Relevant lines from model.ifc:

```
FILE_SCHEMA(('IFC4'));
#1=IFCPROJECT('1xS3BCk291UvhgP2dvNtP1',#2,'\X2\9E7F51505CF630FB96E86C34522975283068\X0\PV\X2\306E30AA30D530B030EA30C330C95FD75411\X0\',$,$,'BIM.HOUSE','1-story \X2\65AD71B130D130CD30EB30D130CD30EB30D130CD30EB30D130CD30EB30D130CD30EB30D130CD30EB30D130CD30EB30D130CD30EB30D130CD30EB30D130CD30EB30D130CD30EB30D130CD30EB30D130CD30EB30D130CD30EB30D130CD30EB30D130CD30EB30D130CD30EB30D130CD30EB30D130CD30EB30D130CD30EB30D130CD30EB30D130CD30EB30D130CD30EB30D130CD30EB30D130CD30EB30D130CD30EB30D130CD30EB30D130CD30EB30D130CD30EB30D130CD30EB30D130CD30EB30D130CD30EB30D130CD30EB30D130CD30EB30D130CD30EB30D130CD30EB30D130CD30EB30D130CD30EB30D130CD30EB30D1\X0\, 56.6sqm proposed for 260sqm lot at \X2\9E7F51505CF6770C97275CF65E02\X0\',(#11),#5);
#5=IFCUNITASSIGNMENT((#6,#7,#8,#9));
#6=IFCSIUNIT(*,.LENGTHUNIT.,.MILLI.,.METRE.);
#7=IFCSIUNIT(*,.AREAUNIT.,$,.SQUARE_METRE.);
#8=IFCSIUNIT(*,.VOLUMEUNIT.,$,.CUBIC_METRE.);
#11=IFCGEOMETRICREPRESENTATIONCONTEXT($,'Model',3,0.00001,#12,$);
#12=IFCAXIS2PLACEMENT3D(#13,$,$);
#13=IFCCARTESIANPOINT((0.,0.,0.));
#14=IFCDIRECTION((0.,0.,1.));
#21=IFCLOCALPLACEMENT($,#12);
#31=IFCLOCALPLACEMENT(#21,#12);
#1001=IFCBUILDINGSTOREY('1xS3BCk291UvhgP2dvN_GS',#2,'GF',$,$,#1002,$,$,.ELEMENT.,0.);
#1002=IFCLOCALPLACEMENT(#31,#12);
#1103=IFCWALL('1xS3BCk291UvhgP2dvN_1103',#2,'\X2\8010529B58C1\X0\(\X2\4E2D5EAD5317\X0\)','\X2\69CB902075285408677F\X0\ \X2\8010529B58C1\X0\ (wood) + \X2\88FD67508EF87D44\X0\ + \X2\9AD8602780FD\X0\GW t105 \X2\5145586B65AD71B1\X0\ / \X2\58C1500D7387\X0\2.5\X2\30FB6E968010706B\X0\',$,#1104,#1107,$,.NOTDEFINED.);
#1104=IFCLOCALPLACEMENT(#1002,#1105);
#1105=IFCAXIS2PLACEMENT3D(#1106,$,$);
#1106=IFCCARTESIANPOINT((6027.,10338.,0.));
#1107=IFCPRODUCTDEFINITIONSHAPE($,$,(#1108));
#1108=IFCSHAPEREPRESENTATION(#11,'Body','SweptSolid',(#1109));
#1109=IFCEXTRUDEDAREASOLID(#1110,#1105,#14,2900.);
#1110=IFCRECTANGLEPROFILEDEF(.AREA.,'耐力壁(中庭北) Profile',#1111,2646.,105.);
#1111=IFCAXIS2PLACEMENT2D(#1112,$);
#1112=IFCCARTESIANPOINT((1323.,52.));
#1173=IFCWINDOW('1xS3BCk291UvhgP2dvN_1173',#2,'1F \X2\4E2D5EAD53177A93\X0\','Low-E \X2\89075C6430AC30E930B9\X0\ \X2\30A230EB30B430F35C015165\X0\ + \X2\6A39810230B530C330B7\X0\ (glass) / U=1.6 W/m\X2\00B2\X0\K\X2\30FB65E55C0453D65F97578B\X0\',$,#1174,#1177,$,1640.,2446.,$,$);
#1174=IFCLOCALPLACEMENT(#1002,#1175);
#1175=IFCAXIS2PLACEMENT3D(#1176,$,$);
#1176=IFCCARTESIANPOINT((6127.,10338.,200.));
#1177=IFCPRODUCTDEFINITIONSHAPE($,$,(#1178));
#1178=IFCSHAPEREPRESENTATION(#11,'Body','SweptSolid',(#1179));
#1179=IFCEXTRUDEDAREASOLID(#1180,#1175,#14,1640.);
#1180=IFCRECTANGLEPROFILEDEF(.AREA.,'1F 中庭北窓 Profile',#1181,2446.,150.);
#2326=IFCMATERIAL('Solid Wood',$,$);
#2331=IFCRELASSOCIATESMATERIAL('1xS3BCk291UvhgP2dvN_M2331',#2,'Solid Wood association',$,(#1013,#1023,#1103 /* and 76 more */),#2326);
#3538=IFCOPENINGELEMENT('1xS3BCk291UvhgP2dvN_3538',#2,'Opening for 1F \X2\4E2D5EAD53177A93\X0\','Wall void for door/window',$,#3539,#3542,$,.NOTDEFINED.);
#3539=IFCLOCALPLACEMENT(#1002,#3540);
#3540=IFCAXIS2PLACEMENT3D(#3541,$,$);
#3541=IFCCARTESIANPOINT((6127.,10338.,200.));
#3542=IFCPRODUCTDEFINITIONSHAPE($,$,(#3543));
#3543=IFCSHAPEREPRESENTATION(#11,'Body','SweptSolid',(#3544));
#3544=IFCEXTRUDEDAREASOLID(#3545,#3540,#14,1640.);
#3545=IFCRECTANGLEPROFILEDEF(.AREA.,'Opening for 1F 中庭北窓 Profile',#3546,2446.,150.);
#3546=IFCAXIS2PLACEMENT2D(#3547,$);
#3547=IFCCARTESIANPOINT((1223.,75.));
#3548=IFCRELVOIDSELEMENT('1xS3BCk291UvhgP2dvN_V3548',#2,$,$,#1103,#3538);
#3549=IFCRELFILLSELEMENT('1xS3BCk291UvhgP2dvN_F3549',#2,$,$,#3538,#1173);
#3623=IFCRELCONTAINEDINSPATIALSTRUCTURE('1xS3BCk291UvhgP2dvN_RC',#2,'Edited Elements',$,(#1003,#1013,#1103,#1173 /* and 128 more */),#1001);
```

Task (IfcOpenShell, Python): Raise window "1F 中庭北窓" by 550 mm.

```python
import numpy as np
import ifcopenshell
import ifcopenshell.api.geometry
import ifcopenshell.util.placement
import ifcopenshell.util.unit

model = ifcopenshell.open("model.ifc")
unit_scale = ifcopenshell.util.unit.calculate_unit_scale(model)

window = model.by_guid("1xS3BCk291UvhgP2dvN_1173")
opening = window.FillsVoids[0].RelatingOpeningElement
dz = 0.55 / unit_scale

shift = np.array([0.0, 0.0, dz])
# The window is not placed relative to its opening, so move both.
for product in (opening, window):
    matrix = ifcopenshell.util.placement.get_local_placement(product.ObjectPlacement)
    matrix[:3, 3] += shift
    ifcopenshell.api.geometry.edit_object_placement(model, product=product, matrix=matrix, is_si=False)

print(f"moved by {dz * unit_scale:+.3f} m")

model.write("model_updated.ifc")
```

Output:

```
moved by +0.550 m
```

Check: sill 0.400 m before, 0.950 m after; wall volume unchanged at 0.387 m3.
